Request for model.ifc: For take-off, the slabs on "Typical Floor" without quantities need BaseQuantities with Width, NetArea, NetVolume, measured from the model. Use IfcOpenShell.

First a look at what the model holds.

```python
import ifcopenshell
import ifcopenshell.util.element
import ifcopenshell.util.unit

model = ifcopenshell.open("model.ifc")
print(model.schema)
for unit_type in ("LENGTHUNIT", "AREAUNIT", "VOLUMEUNIT"):
    print(unit_type, ifcopenshell.util.unit.calculate_unit_scale(model, unit_type))
storey = next(s for s in model.by_type("IfcBuildingStorey") if s.Name == "Typical Floor")
slabs = [e for e in ifcopenshell.util.element.get_decomposition(storey) if e.is_a("IfcSlab")]
for e in sorted(slabs, key=lambda e: e.id()):
    print(e.id(), e.is_a(), e.Name, list(ifcopenshell.util.element.get_psets(e, qtos_only=True)), sep=" | ")
```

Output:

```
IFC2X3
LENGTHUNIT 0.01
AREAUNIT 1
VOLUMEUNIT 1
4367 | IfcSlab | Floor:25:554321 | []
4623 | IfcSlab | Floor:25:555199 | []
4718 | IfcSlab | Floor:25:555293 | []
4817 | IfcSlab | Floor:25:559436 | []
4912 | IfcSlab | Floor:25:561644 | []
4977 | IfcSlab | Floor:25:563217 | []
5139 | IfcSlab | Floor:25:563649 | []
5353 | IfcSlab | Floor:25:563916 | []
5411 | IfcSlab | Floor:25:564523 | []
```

```python
import ifcopenshell
import ifcopenshell.api.pset
import ifcopenshell.geom
import ifcopenshell.util.element
import ifcopenshell.util.shape
import ifcopenshell.util.unit

model = ifcopenshell.open("model.ifc")
unit_scale = ifcopenshell.util.unit.calculate_unit_scale(model)
area_scale = ifcopenshell.util.unit.calculate_unit_scale(model, "AREAUNIT")
volume_scale = ifcopenshell.util.unit.calculate_unit_scale(model, "VOLUMEUNIT")
settings = ifcopenshell.geom.settings()

storey = next(s for s in model.by_type("IfcBuildingStorey") if s.Name == "Typical Floor")
slabs = [e for e in ifcopenshell.util.element.get_decomposition(storey) if e.is_a("IfcSlab")]

for e in sorted(slabs, key=lambda e: e.id()):
    if ifcopenshell.util.element.get_psets(e, qtos_only=True, should_inherit=False):
        continue
    # Geometry comes back in metres, in the element's own axes.
    shape = ifcopenshell.geom.create_shape(settings, e)
    values = {
        "Width": ifcopenshell.util.shape.get_z(shape.geometry) / unit_scale,
        "NetArea": ifcopenshell.util.shape.get_footprint_area(shape.geometry) / area_scale,
        "NetVolume": ifcopenshell.util.shape.get_volume(shape.geometry) / volume_scale,
    }
    qto = ifcopenshell.api.pset.add_qto(model, product=e, name="BaseQuantities")
    ifcopenshell.api.pset.edit_qto(model, qto=qto, properties=values)
    print(e.id(), {k: round(v, 3) for k, v in values.items()})

model.write("model-out.ifc")
```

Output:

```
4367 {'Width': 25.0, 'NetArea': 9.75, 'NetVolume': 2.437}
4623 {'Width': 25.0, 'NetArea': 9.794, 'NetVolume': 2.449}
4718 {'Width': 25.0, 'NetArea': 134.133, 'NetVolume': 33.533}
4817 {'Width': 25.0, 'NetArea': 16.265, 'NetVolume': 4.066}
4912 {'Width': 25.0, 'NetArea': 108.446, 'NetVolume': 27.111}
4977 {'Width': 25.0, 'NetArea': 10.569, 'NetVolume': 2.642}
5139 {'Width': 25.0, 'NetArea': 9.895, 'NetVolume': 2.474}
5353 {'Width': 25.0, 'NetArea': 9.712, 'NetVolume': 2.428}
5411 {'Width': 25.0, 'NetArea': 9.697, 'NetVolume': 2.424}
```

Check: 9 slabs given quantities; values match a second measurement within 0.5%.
